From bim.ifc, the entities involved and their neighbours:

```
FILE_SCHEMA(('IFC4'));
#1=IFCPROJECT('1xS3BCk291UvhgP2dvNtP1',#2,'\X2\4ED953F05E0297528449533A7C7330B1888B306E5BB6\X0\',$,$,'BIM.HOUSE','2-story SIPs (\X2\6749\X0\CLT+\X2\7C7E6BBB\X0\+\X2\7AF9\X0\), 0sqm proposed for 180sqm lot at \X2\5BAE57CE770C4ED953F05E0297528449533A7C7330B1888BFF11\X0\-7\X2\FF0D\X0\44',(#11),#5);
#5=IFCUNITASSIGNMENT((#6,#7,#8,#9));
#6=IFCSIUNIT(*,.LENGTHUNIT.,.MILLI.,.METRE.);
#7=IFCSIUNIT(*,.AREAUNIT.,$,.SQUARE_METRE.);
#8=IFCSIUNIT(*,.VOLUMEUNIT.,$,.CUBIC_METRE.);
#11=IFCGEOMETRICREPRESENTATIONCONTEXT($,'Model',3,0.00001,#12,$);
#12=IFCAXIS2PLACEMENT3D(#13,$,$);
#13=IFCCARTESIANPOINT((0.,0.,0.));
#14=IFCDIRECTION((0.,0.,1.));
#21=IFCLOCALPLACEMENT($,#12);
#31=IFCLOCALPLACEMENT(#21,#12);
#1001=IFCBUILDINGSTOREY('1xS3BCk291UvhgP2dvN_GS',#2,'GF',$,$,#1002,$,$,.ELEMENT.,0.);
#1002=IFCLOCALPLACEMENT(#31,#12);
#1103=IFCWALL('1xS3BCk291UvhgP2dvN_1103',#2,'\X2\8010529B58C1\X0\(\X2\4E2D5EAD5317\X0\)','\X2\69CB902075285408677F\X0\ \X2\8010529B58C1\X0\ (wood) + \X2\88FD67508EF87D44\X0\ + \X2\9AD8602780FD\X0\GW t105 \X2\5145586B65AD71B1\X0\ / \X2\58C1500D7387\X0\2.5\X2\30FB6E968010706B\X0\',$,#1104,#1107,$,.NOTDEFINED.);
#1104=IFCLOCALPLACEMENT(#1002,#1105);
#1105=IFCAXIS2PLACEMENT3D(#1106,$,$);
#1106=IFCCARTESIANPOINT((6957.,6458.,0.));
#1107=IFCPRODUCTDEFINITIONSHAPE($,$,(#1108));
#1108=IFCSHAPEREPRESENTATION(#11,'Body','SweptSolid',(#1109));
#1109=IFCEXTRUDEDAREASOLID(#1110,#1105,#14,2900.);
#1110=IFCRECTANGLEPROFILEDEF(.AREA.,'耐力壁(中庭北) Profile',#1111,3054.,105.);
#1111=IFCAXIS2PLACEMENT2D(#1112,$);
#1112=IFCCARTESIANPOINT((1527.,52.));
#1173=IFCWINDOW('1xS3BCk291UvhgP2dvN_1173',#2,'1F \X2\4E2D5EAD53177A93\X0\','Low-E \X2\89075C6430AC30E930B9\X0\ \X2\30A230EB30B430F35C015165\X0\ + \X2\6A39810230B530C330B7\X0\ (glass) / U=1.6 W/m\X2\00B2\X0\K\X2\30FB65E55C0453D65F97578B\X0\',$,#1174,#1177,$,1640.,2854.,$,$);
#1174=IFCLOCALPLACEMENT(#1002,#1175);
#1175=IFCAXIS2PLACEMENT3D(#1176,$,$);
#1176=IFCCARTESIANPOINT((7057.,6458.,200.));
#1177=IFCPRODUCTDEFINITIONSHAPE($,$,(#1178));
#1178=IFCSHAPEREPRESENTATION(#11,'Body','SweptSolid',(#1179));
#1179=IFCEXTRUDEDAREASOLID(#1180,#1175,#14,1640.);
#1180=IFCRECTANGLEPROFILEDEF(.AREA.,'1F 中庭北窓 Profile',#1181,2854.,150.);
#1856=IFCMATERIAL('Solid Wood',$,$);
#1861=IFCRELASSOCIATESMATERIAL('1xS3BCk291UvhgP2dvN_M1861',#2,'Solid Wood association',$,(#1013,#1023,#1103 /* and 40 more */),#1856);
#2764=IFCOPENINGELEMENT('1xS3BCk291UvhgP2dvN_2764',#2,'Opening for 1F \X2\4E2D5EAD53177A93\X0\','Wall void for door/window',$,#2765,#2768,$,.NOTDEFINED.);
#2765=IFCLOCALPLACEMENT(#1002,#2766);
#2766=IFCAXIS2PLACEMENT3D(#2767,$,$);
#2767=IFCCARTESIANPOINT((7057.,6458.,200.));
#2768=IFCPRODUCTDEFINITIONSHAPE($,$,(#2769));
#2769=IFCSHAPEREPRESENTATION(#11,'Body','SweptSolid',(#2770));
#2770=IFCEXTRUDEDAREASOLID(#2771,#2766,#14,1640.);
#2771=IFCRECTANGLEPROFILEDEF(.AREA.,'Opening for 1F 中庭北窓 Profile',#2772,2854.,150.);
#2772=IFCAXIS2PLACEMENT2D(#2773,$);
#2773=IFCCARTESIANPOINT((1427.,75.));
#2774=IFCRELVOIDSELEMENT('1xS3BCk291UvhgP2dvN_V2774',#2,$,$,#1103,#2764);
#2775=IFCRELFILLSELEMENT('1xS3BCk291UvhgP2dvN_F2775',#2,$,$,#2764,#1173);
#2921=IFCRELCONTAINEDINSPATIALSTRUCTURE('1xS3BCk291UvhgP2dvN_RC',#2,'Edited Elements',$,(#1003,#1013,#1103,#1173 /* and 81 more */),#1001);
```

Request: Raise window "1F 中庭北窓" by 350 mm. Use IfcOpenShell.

```python
import numpy as np
import ifcopenshell
import ifcopenshell.api.geometry
import ifcopenshell.util.placement
import ifcopenshell.util.unit

model = ifcopenshell.open("bim.ifc")
unit_scale = ifcopenshell.util.unit.calculate_unit_scale(model)

window = model.by_id(1173)
opening = window.FillsVoids[0].RelatingOpeningElement
dz = 0.35 / unit_scale

shift = np.array([0.0, 0.0, dz])
# The window is not placed relative to its opening, so move both.
for product in (opening, window):
    matrix = ifcopenshell.util.placement.get_local_placement(product.ObjectPlacement)
    matrix[:3, 3] += shift
    ifcopenshell.api.geometry.edit_object_placement(model, product=product, matrix=matrix, is_si=False)

print(f"moved by {dz * unit_scale:+.3f} m")

model.write("bim-out.ifc")
```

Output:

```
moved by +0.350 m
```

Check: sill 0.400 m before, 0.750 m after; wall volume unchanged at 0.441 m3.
